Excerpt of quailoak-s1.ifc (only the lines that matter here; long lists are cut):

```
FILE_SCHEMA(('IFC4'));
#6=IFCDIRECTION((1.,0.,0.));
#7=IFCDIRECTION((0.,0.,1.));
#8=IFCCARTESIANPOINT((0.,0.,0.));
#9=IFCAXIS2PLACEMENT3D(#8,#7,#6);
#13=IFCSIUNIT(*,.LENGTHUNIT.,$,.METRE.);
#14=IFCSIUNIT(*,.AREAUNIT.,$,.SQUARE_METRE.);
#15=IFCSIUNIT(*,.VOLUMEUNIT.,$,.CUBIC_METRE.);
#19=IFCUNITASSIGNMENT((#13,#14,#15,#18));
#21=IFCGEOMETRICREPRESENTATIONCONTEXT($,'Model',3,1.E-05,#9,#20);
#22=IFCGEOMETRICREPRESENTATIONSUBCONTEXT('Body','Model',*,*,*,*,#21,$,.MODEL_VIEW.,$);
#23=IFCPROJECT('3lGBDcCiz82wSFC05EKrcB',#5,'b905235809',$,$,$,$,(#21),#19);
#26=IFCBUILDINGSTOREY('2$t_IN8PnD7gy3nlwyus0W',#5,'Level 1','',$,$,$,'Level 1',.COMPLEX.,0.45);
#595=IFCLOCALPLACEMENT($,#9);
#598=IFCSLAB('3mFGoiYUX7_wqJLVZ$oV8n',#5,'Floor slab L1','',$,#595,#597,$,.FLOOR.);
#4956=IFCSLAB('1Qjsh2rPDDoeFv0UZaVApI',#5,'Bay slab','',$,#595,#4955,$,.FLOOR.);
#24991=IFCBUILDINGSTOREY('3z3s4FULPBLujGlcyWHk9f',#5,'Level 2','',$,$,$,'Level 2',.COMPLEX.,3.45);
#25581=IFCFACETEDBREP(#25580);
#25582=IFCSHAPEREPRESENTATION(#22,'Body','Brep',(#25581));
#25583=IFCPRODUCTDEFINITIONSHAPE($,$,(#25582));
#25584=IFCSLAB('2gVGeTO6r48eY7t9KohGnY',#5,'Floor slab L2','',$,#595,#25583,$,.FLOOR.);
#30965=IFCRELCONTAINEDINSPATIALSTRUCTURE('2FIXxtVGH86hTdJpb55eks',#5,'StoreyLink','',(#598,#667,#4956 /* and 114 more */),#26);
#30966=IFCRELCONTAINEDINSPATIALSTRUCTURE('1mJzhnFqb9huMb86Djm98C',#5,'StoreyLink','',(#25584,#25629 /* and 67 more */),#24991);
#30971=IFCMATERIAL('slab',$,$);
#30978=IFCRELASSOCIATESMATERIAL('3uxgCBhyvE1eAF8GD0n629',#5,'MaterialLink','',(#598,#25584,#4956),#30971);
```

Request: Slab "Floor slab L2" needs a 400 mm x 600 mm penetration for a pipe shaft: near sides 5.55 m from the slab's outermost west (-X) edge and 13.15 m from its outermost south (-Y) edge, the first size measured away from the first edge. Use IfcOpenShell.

```python
import numpy as np
import ifcopenshell
import ifcopenshell.api.feature
import ifcopenshell.api.geometry
import ifcopenshell.api.root
import ifcopenshell.geom
import ifcopenshell.util.placement
import ifcopenshell.util.representation
import ifcopenshell.util.shape
import ifcopenshell.util.unit

model = ifcopenshell.open("quailoak-s1.ifc")
unit_scale = ifcopenshell.util.unit.calculate_unit_scale(model)
settings = ifcopenshell.geom.settings()


def volume(element):
    """Net volume in cubic metres, openings subtracted."""
    shape = ifcopenshell.geom.create_shape(settings, element)
    return ifcopenshell.util.shape.get_volume(shape.geometry)


slab = model.by_guid("2gVGeTO6r48eY7t9KohGnY")
before = volume(slab)

# Extent in the slab's own axes, in metres. The edges named are its -X and -Y sides.
slab_shape = ifcopenshell.geom.create_shape(settings, slab)
vertices = ifcopenshell.util.shape.get_vertices(slab_shape.geometry)
x_min, y_min, bottom = vertices.min(axis=0)
top = vertices[:, 2].max()

opening = ifcopenshell.api.root.create_entity(model, ifc_class="IfcOpeningElement", name="Pipe shaft opening", predefined_type="OPENING")
context = ifcopenshell.util.representation.get_context(model, "Model", "Body", "MODEL_VIEW")
width, depth = 0.4, 0.6
outline = [(0.0, 0.0), (width, 0.0), (width, depth), (0.0, depth), (0.0, 0.0)]
# Overshoot both faces by 50 mm so the cut is clean.
shape = ifcopenshell.api.geometry.add_slab_representation(
    model, context=context, depth=top - bottom + 0.1, polyline=outline
)
ifcopenshell.api.geometry.assign_representation(model, product=opening, representation=shape)

matrix = ifcopenshell.util.placement.get_local_placement(slab.ObjectPlacement)
matrix[:, 3] = matrix @ np.append(np.array([x_min + 5.55, y_min + 13.15, bottom - 0.05]) / unit_scale, 1.0)
ifcopenshell.api.geometry.edit_object_placement(model, product=opening, matrix=matrix, is_si=False)
ifcopenshell.api.feature.add_feature(model, feature=opening, element=slab)

after = volume(slab)

print(f"slab volume {before:.3f} -> {after:.3f} m3")

model.write("quailoak-s1_edited.ifc")
```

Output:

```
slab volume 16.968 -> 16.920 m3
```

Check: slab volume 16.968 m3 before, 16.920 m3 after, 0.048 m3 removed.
